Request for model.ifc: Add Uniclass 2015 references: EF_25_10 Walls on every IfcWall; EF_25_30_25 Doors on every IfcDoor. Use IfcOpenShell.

First a look at what the model holds.

```python
import ifcopenshell

model = ifcopenshell.open("model.ifc")
print(model.schema)
print("classifications:", [c.Name for c in model.by_type("IfcClassification")])
for ifc_class in ("IfcDoor", "IfcRoof", "IfcStair", "IfcWall", "IfcWindow"):
    print(ifc_class, len(model.by_type(ifc_class)))
```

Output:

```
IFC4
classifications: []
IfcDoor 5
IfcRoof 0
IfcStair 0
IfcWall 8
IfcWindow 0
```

```python
import ifcopenshell
import ifcopenshell.api.classification

model = ifcopenshell.open("model.ifc")

system = ifcopenshell.api.classification.add_classification(model, classification="Uniclass 2015")

codes = {
    "IfcWall": ("EF_25_10", "Walls"),
    "IfcDoor": ("EF_25_30_25", "Doors"),
}
for ifc_class, (code, name) in codes.items():
    products = model.by_type(ifc_class)
    ifcopenshell.api.classification.add_reference(
        model, products=products, classification=system, identification=code, name=name
    )
    print(code, len(products))

model.write("model_rev.ifc")
```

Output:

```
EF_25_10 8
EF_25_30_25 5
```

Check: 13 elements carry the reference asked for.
